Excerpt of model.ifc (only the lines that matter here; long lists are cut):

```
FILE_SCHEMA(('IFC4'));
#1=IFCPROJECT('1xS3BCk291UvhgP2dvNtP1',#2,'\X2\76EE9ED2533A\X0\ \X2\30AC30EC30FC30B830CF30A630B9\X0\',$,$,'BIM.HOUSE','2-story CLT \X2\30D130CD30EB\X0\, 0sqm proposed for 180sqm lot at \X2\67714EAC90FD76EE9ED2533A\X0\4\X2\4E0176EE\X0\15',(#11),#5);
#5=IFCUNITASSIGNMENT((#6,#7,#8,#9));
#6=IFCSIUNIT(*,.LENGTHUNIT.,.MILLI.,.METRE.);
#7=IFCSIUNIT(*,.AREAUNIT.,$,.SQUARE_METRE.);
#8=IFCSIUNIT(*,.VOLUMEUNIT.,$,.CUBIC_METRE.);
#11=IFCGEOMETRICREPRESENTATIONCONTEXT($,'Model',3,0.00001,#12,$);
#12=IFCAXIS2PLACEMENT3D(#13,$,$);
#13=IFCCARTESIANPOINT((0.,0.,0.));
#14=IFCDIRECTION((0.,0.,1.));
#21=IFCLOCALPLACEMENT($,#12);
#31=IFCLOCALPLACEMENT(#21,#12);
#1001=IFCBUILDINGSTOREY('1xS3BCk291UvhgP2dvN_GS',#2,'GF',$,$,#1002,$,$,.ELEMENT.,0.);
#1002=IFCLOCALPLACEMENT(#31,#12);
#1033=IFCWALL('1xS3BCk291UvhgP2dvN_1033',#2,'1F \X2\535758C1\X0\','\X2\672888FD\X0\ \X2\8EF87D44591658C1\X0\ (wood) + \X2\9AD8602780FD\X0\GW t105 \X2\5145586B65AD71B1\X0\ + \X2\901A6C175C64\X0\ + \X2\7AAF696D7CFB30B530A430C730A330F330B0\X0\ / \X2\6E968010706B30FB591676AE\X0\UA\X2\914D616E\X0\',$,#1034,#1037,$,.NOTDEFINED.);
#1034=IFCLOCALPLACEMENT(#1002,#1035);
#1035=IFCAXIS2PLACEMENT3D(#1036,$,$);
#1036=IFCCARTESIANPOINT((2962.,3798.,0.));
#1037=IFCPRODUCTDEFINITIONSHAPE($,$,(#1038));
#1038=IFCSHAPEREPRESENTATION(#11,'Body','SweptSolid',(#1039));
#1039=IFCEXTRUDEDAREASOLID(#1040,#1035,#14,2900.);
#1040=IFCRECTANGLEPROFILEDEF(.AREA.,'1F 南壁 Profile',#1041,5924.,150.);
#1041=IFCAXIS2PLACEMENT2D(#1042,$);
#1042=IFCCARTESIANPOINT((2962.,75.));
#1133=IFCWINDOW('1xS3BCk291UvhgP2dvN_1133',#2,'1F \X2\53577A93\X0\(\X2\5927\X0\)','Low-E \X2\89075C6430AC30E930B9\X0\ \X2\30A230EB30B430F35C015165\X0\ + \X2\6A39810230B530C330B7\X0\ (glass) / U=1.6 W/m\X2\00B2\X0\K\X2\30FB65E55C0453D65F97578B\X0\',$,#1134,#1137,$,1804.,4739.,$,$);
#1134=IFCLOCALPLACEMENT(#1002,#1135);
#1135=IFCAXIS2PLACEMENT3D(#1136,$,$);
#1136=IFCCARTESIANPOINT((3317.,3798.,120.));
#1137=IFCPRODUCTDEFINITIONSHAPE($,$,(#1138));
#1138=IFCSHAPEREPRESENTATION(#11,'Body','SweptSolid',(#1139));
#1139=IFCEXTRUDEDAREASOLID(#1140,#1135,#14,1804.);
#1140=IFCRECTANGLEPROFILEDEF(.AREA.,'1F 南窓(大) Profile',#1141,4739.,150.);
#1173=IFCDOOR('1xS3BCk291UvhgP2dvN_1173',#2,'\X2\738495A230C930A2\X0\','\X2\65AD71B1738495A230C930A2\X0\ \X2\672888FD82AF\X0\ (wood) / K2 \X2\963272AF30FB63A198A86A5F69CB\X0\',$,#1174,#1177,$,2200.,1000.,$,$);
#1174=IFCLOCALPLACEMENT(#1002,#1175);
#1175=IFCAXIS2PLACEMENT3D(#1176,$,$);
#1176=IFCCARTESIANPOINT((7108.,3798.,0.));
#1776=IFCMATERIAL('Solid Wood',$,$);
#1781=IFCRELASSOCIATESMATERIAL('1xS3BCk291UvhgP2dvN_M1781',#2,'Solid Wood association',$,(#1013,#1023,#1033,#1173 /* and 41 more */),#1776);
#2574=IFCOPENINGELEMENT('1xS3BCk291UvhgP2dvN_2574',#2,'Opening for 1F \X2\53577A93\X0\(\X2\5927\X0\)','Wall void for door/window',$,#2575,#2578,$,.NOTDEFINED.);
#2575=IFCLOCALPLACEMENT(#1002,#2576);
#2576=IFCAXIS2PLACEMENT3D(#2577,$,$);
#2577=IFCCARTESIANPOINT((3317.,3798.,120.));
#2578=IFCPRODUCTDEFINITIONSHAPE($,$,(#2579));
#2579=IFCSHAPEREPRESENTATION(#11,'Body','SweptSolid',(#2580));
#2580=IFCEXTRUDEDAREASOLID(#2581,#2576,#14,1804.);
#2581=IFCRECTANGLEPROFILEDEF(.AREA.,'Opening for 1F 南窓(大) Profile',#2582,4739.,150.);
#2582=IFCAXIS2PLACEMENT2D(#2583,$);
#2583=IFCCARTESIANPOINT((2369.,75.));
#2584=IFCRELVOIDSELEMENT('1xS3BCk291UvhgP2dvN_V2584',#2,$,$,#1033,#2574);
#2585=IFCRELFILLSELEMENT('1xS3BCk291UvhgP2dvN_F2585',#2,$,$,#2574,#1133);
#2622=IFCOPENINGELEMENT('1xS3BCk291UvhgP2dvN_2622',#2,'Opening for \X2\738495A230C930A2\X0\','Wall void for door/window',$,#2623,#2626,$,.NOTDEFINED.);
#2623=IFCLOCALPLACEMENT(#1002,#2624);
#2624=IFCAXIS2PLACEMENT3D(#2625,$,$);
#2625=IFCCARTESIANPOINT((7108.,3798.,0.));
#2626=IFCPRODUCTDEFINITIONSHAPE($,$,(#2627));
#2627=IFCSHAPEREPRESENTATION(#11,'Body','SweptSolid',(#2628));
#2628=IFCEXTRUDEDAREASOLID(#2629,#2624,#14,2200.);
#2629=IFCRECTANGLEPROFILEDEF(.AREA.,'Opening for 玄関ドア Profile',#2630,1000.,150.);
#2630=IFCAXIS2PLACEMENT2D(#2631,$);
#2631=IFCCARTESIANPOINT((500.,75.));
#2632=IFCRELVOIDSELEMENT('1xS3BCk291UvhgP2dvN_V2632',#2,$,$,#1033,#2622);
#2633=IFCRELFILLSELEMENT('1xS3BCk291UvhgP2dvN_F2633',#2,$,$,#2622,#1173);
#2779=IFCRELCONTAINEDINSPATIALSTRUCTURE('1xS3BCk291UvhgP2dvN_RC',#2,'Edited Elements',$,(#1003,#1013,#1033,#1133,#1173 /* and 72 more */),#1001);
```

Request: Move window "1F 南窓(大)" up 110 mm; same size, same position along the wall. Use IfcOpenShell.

```python
import numpy as np
import ifcopenshell
import ifcopenshell.api.geometry
import ifcopenshell.util.placement
import ifcopenshell.util.unit

model = ifcopenshell.open("model.ifc")
unit_scale = ifcopenshell.util.unit.calculate_unit_scale(model)

window = model.by_guid("1xS3BCk291UvhgP2dvN_1133")
opening = window.FillsVoids[0].RelatingOpeningElement
dz = 0.11 / unit_scale

shift = np.array([0.0, 0.0, dz])
# The window is not placed relative to its opening, so move both.
for product in (opening, window):
    matrix = ifcopenshell.util.placement.get_local_placement(product.ObjectPlacement)
    matrix[:3, 3] += shift
    ifcopenshell.api.geometry.edit_object_placement(model, product=product, matrix=matrix, is_si=False)

print(f"moved by {dz * unit_scale:+.3f} m")

model.write("model_edited.ifc")
```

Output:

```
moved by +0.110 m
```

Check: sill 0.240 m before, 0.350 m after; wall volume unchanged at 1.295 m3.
